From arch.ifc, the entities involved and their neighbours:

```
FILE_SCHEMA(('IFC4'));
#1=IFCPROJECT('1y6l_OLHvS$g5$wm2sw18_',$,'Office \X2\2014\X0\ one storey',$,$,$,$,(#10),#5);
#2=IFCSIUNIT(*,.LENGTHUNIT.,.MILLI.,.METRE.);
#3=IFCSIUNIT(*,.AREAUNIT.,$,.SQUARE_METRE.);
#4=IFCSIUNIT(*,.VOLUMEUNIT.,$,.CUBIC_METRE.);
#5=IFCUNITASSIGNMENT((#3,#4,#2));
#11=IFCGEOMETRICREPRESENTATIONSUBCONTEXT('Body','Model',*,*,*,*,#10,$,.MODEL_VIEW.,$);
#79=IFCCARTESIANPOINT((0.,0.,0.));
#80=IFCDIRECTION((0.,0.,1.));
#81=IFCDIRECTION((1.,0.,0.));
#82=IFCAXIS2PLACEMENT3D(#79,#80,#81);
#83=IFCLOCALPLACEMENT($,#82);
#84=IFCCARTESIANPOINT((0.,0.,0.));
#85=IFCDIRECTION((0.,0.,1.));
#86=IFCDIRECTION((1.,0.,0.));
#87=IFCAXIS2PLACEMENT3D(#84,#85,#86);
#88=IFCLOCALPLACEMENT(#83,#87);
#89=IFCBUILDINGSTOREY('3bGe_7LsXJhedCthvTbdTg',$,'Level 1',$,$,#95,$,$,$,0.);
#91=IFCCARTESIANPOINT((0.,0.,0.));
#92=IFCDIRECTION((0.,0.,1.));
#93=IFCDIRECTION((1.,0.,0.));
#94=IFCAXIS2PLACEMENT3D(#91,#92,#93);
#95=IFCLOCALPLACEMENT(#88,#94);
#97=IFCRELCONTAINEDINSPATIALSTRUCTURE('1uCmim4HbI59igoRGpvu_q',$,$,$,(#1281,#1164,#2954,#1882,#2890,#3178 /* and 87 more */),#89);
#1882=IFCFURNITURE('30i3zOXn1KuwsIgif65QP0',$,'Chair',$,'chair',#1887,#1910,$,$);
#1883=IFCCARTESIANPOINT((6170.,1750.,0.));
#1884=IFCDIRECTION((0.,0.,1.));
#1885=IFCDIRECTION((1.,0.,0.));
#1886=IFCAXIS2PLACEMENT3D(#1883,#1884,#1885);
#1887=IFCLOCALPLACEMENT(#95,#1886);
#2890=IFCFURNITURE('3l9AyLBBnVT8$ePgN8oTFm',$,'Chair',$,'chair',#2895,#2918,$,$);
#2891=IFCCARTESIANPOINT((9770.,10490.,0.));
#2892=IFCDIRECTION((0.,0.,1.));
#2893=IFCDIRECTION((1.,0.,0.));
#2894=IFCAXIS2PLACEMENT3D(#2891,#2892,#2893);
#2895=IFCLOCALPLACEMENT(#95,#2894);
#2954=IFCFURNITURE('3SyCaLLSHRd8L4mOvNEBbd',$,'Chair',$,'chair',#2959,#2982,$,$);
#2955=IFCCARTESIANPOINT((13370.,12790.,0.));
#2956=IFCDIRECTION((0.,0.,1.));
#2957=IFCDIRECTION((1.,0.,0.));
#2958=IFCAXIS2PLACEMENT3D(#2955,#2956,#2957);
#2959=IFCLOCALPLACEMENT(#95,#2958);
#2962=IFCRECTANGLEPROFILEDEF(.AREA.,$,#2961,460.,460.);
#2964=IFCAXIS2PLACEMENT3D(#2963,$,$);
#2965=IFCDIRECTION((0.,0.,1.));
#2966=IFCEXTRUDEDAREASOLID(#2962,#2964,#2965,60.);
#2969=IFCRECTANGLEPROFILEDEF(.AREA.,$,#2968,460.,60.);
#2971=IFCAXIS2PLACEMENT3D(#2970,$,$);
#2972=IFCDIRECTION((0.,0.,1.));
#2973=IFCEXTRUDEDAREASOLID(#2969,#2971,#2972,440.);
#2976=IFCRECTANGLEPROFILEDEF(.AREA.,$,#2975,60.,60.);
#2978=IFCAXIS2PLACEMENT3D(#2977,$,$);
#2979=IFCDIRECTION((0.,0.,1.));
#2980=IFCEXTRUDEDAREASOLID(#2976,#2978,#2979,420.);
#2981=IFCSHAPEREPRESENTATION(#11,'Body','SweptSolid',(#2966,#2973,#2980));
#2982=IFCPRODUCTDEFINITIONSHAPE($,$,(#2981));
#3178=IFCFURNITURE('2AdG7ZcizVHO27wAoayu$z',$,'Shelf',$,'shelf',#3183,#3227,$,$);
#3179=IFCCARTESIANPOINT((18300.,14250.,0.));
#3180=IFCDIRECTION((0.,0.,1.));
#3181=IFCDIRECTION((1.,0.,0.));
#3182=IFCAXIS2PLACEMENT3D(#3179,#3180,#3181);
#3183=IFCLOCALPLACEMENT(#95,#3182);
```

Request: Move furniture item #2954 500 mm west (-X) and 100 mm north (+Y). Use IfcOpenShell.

```python
import ifcopenshell
import ifcopenshell.api.geometry
import ifcopenshell.util.placement
import ifcopenshell.util.unit

model = ifcopenshell.open("arch.ifc")
unit_scale = ifcopenshell.util.unit.calculate_unit_scale(model)

item = model.by_guid("3SyCaLLSHRd8L4mOvNEBbd")
matrix = ifcopenshell.util.placement.get_local_placement(item.ObjectPlacement)
matrix[0, 3] -= 0.5 / unit_scale
matrix[1, 3] += 0.1 / unit_scale
ifcopenshell.api.geometry.edit_object_placement(model, product=item, matrix=matrix, is_si=False)

print(ifcopenshell.util.placement.get_local_placement(item.ObjectPlacement).round(3) + 0.0)

model.write("arch_edited.ifc")
```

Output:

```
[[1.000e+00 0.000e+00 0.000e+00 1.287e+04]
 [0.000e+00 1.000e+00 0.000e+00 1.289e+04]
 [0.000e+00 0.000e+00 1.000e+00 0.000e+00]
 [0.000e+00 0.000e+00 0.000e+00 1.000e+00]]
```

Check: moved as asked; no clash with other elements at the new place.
